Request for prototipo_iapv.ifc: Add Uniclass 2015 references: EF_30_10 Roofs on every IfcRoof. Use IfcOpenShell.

First a look at what the model holds.

```python
import ifcopenshell

model = ifcopenshell.open("prototipo_iapv.ifc")
print(model.schema)
print("classifications:", [c.Name for c in model.by_type("IfcClassification")])
for ifc_class in ("IfcDoor", "IfcRoof", "IfcStair", "IfcWall", "IfcWindow"):
    print(ifc_class, len(model.by_type(ifc_class)))
```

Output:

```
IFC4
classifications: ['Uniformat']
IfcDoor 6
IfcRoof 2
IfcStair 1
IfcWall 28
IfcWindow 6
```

```python
import ifcopenshell
import ifcopenshell.api.classification

model = ifcopenshell.open("prototipo_iapv.ifc")

system = ifcopenshell.api.classification.add_classification(model, classification="Uniclass 2015")

codes = {
    "IfcRoof": ("EF_30_10", "Roofs"),
}
for ifc_class, (code, name) in codes.items():
    products = model.by_type(ifc_class)
    ifcopenshell.api.classification.add_reference(
        model, products=products, classification=system, identification=code, name=name
    )
    print(code, len(products))

model.write("prototipo_iapv-out.ifc")
```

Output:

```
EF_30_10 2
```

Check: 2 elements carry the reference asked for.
